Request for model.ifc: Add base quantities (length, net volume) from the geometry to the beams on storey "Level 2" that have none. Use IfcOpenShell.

First a look at what the model holds.

```python
import ifcopenshell
import ifcopenshell.util.element
import ifcopenshell.util.unit

model = ifcopenshell.open("model.ifc")
print(model.schema)
for unit_type in ("LENGTHUNIT", "AREAUNIT", "VOLUMEUNIT"):
    print(unit_type, ifcopenshell.util.unit.calculate_unit_scale(model, unit_type))
storey = next(s for s in model.by_type("IfcBuildingStorey") if s.Name == "Level 2")
beams = [e for e in ifcopenshell.util.element.get_decomposition(storey) if e.is_a("IfcBeam")]
for e in sorted(beams, key=lambda e: e.id()):
    print(e.id(), e.is_a(), e.Name, list(ifcopenshell.util.element.get_psets(e, qtos_only=True)), sep=" | ")
```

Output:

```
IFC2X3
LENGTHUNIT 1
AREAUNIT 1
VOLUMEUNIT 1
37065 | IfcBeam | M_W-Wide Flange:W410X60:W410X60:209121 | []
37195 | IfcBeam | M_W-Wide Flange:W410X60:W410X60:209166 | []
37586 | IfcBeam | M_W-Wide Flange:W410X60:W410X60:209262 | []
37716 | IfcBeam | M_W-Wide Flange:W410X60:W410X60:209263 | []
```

```python
import ifcopenshell
import ifcopenshell.api.pset
import ifcopenshell.geom
import ifcopenshell.util.element
import ifcopenshell.util.shape
import ifcopenshell.util.unit

model = ifcopenshell.open("model.ifc")
unit_scale = ifcopenshell.util.unit.calculate_unit_scale(model)
volume_scale = ifcopenshell.util.unit.calculate_unit_scale(model, "VOLUMEUNIT")
settings = ifcopenshell.geom.settings()

storey = next(s for s in model.by_type("IfcBuildingStorey") if s.Name == "Level 2")
beams = [e for e in ifcopenshell.util.element.get_decomposition(storey) if e.is_a("IfcBeam")]

for e in sorted(beams, key=lambda e: e.id()):
    if ifcopenshell.util.element.get_psets(e, qtos_only=True, should_inherit=False):
        continue
    # Geometry comes back in metres, in the element's own axes.
    shape = ifcopenshell.geom.create_shape(settings, e)
    values = {
        "Length": ifcopenshell.util.shape.get_max_xyz(shape.geometry) / unit_scale,
        "NetVolume": ifcopenshell.util.shape.get_volume(shape.geometry) / volume_scale,
    }
    qto = ifcopenshell.api.pset.add_qto(model, product=e, name="BaseQuantities")
    ifcopenshell.api.pset.edit_qto(model, qto=qto, properties=values)
    print(e.id(), {k: round(v, 3) for k, v in values.items()})

model.write("model-out.ifc")
```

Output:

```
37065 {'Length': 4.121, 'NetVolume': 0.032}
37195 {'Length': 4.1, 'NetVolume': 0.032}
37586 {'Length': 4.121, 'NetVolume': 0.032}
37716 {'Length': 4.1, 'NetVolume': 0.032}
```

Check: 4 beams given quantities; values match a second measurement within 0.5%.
